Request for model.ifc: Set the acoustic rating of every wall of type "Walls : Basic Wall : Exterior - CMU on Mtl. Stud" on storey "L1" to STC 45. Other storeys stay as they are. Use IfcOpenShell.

First a look at what the model holds.

```python
import ifcopenshell
import ifcopenshell.util.element

model = ifcopenshell.open("model.ifc")
print(model.schema)
storey = next(s for s in model.by_type("IfcBuildingStorey") if s.Name == "L1")
walls = [e for e in ifcopenshell.util.element.get_decomposition(storey) if e.is_a("IfcWall")]
seen = {}
for e in walls:
    element_type = ifcopenshell.util.element.get_type(e)
    key = (element_type.Name if element_type != e and element_type else None, ifcopenshell.util.element.get_pset(e, "Pset_WallCommon", "AcousticRating"))
    seen[key] = seen.get(key, 0) + 1
for (name, value), count in sorted(seen.items(), key=str):
    print(count, "x", name, "|", value)
```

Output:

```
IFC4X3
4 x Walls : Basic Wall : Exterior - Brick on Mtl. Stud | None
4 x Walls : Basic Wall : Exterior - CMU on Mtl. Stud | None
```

```python
import ifcopenshell
import ifcopenshell.api.pset
import ifcopenshell.util.element

model = ifcopenshell.open("model.ifc")

storey = next(s for s in model.by_type("IfcBuildingStorey") if s.Name == "L1")
walls = [e for e in ifcopenshell.util.element.get_decomposition(storey) if e.is_a("IfcWall")]

count = 0
for e in walls:
    element_type = ifcopenshell.util.element.get_type(e)
    if element_type in (None, e) or element_type.Name != "Walls : Basic Wall : Exterior - CMU on Mtl. Stud":
        continue
    # add_pset returns the element's existing set when there is one.
    pset = ifcopenshell.api.pset.add_pset(model, product=e, name="Pset_WallCommon")
    ifcopenshell.api.pset.edit_pset(model, pset=pset, properties={"AcousticRating": "STC 45"})
    count += 1

print(count, "walls updated")

model.write("model-out.ifc")
```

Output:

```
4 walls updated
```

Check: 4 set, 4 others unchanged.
